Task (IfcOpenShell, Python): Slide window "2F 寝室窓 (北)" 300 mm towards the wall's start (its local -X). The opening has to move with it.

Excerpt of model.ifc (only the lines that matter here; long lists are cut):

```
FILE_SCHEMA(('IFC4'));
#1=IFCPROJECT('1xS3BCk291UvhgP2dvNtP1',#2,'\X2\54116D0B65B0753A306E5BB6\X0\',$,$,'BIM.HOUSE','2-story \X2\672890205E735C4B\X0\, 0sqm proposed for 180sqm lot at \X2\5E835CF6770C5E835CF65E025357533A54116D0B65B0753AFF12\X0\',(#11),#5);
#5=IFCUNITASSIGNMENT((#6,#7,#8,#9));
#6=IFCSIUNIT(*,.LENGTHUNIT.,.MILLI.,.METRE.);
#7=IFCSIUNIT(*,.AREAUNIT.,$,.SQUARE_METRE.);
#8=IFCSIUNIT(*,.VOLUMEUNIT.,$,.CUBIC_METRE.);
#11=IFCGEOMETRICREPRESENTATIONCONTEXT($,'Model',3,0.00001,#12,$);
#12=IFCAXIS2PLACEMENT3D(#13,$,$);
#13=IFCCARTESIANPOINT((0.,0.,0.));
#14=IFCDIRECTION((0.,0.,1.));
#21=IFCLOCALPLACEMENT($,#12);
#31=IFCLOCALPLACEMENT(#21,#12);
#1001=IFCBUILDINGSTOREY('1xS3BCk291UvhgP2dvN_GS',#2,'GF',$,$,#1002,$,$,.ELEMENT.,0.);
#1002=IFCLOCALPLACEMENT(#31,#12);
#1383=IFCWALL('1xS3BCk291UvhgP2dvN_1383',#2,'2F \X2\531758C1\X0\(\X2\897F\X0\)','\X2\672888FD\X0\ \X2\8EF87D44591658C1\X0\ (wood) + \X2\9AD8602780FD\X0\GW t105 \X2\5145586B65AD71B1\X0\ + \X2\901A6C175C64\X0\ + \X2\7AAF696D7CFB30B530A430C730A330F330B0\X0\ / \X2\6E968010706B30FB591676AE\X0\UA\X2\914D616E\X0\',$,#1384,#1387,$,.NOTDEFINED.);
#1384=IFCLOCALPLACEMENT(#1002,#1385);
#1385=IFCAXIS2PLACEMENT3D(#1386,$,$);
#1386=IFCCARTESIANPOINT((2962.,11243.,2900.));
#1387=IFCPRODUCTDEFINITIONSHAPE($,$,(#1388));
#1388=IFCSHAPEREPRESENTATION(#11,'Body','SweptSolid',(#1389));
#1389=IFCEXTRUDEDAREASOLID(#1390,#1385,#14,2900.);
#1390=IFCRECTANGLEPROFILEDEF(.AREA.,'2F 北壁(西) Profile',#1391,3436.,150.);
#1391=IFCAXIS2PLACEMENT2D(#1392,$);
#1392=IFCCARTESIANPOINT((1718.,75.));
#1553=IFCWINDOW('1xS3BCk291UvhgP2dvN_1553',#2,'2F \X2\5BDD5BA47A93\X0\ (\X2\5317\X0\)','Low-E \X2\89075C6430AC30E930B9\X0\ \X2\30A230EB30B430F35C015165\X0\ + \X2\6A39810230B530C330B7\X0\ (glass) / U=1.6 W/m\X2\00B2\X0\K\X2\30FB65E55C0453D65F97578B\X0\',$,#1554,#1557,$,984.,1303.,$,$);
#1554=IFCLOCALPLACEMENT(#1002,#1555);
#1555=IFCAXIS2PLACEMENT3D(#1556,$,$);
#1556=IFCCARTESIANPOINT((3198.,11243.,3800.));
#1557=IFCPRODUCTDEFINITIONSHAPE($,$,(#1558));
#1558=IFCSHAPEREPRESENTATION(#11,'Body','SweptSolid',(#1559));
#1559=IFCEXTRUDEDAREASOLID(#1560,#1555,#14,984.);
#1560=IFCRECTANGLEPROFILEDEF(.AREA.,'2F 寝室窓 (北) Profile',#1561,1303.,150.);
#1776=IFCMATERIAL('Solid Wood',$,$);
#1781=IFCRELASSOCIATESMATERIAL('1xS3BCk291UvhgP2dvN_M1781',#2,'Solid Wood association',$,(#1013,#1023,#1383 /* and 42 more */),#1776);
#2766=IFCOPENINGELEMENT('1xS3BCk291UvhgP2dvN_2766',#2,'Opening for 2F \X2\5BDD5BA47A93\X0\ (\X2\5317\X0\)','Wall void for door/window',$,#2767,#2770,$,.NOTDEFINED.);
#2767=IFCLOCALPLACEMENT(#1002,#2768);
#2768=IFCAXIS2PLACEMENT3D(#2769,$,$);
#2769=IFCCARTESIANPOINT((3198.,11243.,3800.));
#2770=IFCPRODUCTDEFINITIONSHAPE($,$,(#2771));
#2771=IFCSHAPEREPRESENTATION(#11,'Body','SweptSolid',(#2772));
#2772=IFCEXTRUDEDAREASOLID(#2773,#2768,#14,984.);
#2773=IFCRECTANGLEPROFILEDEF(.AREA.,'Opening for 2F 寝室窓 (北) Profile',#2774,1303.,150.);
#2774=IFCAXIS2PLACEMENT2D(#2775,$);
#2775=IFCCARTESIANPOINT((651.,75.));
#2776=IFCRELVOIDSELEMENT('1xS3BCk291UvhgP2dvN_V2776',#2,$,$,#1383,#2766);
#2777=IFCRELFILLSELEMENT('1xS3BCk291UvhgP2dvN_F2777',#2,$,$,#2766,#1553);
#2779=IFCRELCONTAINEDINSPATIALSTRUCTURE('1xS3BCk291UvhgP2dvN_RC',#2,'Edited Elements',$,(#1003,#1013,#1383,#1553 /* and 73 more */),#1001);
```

```python
import ifcopenshell
import ifcopenshell.api.geometry
import ifcopenshell.util.placement
import ifcopenshell.util.unit

model = ifcopenshell.open("model.ifc")
unit_scale = ifcopenshell.util.unit.calculate_unit_scale(model)

window = model.by_guid("1xS3BCk291UvhgP2dvN_1553")
opening = window.FillsVoids[0].RelatingOpeningElement
wall = opening.VoidsElements[0].RelatingBuildingElement

wall_matrix = ifcopenshell.util.placement.get_local_placement(wall.ObjectPlacement)
shift = wall_matrix[:3, 0] * -0.3 / unit_scale
before = ifcopenshell.util.placement.get_local_placement(window.ObjectPlacement)[:3, 3].copy()

# The window is not placed relative to its opening, so move both.
for product in (opening, window):
    matrix = ifcopenshell.util.placement.get_local_placement(product.ObjectPlacement)
    matrix[:3, 3] += shift
    ifcopenshell.api.geometry.edit_object_placement(model, product=product, matrix=matrix, is_si=False)

after = ifcopenshell.util.placement.get_local_placement(window.ObjectPlacement)[:3, 3]
print("window moved by", (after - before).round(3) + 0.0)

model.write("model_v2.ifc")
```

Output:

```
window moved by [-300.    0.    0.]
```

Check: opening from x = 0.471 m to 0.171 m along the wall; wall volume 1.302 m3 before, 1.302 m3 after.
